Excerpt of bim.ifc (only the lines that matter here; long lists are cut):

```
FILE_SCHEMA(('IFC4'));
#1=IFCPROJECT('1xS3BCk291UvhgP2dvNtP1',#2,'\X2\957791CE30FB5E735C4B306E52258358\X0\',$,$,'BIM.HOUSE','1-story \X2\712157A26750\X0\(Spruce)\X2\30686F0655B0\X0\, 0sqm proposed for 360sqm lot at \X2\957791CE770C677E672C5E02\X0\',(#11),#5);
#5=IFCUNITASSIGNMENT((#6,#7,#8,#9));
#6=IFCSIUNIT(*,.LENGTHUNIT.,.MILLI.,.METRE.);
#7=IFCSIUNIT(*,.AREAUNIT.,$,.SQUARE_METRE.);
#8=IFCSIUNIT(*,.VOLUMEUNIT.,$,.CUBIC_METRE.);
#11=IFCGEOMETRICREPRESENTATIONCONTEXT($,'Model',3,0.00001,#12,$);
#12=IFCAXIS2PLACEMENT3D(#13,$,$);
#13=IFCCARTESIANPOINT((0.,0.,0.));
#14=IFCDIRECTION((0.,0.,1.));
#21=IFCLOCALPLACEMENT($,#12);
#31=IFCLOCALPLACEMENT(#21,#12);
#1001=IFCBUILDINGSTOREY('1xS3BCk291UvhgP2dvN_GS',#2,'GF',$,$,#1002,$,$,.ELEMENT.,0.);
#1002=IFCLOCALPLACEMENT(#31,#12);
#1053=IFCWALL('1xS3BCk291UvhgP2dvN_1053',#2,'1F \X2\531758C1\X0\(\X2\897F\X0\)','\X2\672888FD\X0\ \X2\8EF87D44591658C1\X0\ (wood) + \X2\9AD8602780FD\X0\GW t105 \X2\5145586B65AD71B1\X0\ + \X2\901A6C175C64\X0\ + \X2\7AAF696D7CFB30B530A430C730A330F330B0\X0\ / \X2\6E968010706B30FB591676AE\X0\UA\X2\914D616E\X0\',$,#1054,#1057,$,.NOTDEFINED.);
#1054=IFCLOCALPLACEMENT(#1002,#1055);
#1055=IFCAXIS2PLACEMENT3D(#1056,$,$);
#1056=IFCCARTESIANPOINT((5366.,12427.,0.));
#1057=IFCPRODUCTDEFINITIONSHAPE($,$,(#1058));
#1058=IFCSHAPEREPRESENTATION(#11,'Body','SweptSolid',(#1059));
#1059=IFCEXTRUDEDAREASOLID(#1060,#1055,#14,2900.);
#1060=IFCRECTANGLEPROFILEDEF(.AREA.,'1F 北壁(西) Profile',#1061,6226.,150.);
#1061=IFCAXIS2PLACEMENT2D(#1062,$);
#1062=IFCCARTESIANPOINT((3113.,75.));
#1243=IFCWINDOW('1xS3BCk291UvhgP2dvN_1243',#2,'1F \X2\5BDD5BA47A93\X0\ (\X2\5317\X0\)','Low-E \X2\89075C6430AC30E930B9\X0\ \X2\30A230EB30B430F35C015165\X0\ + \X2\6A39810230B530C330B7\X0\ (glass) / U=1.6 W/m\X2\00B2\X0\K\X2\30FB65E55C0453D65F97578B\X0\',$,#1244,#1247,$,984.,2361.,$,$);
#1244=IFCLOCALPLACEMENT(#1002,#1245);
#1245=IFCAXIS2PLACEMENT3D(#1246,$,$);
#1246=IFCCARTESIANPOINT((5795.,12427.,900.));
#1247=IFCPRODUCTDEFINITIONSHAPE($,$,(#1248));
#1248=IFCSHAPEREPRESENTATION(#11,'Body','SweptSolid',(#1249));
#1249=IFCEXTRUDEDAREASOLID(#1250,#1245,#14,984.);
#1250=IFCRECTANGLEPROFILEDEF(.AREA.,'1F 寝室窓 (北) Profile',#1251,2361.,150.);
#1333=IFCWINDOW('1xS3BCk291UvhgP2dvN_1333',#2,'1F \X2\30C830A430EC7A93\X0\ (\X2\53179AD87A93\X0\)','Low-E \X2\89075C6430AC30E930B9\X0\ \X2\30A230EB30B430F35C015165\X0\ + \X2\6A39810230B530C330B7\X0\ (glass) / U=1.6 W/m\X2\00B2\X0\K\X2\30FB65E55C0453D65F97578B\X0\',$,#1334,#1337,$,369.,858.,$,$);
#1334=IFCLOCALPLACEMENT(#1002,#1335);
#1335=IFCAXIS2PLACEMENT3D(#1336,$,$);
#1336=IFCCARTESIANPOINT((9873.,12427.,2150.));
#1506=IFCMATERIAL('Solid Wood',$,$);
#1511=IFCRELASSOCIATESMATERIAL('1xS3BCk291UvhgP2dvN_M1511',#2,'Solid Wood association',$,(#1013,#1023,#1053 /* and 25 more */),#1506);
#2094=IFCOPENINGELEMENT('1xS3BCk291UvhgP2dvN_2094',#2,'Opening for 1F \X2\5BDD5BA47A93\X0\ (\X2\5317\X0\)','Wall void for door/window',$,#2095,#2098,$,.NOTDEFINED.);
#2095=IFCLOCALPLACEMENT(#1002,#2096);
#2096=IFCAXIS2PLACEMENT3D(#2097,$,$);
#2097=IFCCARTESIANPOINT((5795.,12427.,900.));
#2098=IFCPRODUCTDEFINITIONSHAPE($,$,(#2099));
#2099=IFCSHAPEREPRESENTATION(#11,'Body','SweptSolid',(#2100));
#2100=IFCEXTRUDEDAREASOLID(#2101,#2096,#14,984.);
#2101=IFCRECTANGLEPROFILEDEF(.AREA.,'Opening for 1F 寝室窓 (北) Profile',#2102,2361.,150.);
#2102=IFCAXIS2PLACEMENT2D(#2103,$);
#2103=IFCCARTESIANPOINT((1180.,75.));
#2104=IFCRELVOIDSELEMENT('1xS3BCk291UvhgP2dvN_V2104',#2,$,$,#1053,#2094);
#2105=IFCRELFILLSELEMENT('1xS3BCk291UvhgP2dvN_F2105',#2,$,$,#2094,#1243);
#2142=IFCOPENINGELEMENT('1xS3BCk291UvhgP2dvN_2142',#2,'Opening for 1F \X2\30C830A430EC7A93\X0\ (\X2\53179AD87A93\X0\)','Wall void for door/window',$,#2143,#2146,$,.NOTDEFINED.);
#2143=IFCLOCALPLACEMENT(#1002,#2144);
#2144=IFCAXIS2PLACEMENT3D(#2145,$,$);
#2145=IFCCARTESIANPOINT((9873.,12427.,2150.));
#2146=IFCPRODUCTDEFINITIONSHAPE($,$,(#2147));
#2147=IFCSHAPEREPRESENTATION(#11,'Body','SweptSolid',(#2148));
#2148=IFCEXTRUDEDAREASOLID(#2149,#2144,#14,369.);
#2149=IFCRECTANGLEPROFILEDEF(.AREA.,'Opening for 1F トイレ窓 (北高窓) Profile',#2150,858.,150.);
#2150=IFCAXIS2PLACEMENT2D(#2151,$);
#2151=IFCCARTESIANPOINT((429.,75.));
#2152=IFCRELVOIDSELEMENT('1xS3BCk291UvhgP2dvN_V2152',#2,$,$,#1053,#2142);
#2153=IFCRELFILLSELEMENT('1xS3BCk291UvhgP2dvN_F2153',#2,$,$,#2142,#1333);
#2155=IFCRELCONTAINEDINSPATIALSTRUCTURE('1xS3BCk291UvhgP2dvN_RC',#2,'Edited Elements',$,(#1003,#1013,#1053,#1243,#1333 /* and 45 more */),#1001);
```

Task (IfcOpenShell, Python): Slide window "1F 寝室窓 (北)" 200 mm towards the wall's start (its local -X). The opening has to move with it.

```python
import ifcopenshell
import ifcopenshell.api.geometry
import ifcopenshell.util.placement
import ifcopenshell.util.unit

model = ifcopenshell.open("bim.ifc")
unit_scale = ifcopenshell.util.unit.calculate_unit_scale(model)

window = model.by_guid("1xS3BCk291UvhgP2dvN_1243")
opening = window.FillsVoids[0].RelatingOpeningElement
wall = opening.VoidsElements[0].RelatingBuildingElement

wall_matrix = ifcopenshell.util.placement.get_local_placement(wall.ObjectPlacement)
shift = wall_matrix[:3, 0] * -0.2 / unit_scale
before = ifcopenshell.util.placement.get_local_placement(window.ObjectPlacement)[:3, 3].copy()

# The window is not placed relative to its opening, so move both.
for product in (opening, window):
    matrix = ifcopenshell.util.placement.get_local_placement(product.ObjectPlacement)
    matrix[:3, 3] += shift
    ifcopenshell.api.geometry.edit_object_placement(model, product=product, matrix=matrix, is_si=False)

after = ifcopenshell.util.placement.get_local_placement(window.ObjectPlacement)[:3, 3]
print("window moved by", (after - before).round(3) + 0.0)

model.write("bim_updated.ifc")
```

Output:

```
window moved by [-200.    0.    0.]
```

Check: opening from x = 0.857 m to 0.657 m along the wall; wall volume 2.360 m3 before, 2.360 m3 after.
